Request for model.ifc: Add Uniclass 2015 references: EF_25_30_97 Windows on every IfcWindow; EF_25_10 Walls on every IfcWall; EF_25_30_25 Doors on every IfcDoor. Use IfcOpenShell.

First a look at what the model holds.

```python
import ifcopenshell

model = ifcopenshell.open("model.ifc")
print(model.schema)
print("classifications:", [c.Name for c in model.by_type("IfcClassification")])
for ifc_class in ("IfcDoor", "IfcRoof", "IfcStair", "IfcWall", "IfcWindow"):
    print(ifc_class, len(model.by_type(ifc_class)))
```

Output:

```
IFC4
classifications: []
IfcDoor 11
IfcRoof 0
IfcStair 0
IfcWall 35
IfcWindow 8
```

```python
import ifcopenshell
import ifcopenshell.api.classification

model = ifcopenshell.open("model.ifc")

system = ifcopenshell.api.classification.add_classification(model, classification="Uniclass 2015")

codes = {
    "IfcWindow": ("EF_25_30_97", "Windows"),
    "IfcWall": ("EF_25_10", "Walls"),
    "IfcDoor": ("EF_25_30_25", "Doors"),
}
for ifc_class, (code, name) in codes.items():
    products = model.by_type(ifc_class)
    ifcopenshell.api.classification.add_reference(
        model, products=products, classification=system, identification=code, name=name
    )
    print(code, len(products))

model.write("model_edited.ifc")
```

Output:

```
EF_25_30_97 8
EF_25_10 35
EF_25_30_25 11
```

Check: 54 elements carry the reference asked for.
